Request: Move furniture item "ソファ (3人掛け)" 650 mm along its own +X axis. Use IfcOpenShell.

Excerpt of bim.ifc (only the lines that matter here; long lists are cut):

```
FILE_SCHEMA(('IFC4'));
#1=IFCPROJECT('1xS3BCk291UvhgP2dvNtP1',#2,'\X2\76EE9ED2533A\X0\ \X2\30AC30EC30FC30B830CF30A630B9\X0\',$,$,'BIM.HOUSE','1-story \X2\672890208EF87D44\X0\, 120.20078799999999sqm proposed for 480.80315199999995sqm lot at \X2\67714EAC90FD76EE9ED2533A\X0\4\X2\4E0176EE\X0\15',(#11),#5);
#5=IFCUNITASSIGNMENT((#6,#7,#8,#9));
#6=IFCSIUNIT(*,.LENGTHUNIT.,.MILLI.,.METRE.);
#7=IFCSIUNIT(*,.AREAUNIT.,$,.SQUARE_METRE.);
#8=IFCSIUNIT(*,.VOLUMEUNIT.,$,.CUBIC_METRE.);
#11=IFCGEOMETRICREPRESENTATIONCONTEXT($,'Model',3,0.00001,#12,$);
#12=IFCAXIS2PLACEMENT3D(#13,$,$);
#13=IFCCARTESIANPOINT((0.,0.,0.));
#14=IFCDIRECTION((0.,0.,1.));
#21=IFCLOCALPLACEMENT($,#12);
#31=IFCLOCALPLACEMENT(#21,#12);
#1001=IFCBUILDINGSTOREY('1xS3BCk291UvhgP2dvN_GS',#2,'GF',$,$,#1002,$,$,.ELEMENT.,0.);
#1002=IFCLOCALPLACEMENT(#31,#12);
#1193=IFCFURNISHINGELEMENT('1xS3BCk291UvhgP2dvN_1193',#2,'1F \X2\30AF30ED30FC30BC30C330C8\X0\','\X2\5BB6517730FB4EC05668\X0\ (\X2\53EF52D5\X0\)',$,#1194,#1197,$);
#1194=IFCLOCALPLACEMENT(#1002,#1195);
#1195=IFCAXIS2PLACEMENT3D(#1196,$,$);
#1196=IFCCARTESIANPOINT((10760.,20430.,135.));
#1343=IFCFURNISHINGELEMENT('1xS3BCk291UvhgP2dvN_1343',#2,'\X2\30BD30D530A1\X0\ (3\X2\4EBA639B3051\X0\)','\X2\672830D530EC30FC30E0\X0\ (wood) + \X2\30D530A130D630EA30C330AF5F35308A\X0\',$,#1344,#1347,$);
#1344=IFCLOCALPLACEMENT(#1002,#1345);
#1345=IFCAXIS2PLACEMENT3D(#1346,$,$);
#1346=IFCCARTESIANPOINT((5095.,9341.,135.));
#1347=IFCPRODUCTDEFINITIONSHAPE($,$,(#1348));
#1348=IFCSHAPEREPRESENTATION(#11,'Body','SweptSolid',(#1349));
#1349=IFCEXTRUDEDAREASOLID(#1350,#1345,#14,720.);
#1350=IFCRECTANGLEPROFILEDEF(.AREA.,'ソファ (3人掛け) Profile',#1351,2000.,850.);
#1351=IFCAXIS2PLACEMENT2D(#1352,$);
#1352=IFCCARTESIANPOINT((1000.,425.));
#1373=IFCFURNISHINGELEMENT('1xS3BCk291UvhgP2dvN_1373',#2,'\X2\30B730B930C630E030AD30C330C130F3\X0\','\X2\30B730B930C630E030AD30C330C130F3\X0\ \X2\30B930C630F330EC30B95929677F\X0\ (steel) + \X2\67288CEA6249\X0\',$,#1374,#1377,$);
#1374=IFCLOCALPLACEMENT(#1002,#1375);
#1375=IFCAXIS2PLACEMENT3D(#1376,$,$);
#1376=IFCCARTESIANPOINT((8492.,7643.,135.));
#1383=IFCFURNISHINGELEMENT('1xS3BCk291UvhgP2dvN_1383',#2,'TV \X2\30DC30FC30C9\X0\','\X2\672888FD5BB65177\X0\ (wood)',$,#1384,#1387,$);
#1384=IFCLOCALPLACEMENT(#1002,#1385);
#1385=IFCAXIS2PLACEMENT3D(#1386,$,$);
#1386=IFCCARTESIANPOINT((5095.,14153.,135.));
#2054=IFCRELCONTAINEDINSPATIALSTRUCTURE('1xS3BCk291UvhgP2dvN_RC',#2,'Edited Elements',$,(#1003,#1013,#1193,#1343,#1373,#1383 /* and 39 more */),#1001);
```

```python
import ifcopenshell
import ifcopenshell.api.geometry
import ifcopenshell.util.placement
import ifcopenshell.util.unit

model = ifcopenshell.open("bim.ifc")
unit_scale = ifcopenshell.util.unit.calculate_unit_scale(model)

item = model.by_guid("1xS3BCk291UvhgP2dvN_1343")
matrix = ifcopenshell.util.placement.get_local_placement(item.ObjectPlacement)
matrix[:3, 3] += matrix[:3, 0] * 0.65 / unit_scale
ifcopenshell.api.geometry.edit_object_placement(model, product=item, matrix=matrix, is_si=False)

print(ifcopenshell.util.placement.get_local_placement(item.ObjectPlacement).round(3) + 0.0)

model.write("bim_updated.ifc")
```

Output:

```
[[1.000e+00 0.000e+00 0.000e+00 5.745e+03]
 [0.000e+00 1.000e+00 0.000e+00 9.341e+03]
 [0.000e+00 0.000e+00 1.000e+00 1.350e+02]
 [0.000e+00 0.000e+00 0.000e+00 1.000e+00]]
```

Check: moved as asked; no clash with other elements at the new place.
